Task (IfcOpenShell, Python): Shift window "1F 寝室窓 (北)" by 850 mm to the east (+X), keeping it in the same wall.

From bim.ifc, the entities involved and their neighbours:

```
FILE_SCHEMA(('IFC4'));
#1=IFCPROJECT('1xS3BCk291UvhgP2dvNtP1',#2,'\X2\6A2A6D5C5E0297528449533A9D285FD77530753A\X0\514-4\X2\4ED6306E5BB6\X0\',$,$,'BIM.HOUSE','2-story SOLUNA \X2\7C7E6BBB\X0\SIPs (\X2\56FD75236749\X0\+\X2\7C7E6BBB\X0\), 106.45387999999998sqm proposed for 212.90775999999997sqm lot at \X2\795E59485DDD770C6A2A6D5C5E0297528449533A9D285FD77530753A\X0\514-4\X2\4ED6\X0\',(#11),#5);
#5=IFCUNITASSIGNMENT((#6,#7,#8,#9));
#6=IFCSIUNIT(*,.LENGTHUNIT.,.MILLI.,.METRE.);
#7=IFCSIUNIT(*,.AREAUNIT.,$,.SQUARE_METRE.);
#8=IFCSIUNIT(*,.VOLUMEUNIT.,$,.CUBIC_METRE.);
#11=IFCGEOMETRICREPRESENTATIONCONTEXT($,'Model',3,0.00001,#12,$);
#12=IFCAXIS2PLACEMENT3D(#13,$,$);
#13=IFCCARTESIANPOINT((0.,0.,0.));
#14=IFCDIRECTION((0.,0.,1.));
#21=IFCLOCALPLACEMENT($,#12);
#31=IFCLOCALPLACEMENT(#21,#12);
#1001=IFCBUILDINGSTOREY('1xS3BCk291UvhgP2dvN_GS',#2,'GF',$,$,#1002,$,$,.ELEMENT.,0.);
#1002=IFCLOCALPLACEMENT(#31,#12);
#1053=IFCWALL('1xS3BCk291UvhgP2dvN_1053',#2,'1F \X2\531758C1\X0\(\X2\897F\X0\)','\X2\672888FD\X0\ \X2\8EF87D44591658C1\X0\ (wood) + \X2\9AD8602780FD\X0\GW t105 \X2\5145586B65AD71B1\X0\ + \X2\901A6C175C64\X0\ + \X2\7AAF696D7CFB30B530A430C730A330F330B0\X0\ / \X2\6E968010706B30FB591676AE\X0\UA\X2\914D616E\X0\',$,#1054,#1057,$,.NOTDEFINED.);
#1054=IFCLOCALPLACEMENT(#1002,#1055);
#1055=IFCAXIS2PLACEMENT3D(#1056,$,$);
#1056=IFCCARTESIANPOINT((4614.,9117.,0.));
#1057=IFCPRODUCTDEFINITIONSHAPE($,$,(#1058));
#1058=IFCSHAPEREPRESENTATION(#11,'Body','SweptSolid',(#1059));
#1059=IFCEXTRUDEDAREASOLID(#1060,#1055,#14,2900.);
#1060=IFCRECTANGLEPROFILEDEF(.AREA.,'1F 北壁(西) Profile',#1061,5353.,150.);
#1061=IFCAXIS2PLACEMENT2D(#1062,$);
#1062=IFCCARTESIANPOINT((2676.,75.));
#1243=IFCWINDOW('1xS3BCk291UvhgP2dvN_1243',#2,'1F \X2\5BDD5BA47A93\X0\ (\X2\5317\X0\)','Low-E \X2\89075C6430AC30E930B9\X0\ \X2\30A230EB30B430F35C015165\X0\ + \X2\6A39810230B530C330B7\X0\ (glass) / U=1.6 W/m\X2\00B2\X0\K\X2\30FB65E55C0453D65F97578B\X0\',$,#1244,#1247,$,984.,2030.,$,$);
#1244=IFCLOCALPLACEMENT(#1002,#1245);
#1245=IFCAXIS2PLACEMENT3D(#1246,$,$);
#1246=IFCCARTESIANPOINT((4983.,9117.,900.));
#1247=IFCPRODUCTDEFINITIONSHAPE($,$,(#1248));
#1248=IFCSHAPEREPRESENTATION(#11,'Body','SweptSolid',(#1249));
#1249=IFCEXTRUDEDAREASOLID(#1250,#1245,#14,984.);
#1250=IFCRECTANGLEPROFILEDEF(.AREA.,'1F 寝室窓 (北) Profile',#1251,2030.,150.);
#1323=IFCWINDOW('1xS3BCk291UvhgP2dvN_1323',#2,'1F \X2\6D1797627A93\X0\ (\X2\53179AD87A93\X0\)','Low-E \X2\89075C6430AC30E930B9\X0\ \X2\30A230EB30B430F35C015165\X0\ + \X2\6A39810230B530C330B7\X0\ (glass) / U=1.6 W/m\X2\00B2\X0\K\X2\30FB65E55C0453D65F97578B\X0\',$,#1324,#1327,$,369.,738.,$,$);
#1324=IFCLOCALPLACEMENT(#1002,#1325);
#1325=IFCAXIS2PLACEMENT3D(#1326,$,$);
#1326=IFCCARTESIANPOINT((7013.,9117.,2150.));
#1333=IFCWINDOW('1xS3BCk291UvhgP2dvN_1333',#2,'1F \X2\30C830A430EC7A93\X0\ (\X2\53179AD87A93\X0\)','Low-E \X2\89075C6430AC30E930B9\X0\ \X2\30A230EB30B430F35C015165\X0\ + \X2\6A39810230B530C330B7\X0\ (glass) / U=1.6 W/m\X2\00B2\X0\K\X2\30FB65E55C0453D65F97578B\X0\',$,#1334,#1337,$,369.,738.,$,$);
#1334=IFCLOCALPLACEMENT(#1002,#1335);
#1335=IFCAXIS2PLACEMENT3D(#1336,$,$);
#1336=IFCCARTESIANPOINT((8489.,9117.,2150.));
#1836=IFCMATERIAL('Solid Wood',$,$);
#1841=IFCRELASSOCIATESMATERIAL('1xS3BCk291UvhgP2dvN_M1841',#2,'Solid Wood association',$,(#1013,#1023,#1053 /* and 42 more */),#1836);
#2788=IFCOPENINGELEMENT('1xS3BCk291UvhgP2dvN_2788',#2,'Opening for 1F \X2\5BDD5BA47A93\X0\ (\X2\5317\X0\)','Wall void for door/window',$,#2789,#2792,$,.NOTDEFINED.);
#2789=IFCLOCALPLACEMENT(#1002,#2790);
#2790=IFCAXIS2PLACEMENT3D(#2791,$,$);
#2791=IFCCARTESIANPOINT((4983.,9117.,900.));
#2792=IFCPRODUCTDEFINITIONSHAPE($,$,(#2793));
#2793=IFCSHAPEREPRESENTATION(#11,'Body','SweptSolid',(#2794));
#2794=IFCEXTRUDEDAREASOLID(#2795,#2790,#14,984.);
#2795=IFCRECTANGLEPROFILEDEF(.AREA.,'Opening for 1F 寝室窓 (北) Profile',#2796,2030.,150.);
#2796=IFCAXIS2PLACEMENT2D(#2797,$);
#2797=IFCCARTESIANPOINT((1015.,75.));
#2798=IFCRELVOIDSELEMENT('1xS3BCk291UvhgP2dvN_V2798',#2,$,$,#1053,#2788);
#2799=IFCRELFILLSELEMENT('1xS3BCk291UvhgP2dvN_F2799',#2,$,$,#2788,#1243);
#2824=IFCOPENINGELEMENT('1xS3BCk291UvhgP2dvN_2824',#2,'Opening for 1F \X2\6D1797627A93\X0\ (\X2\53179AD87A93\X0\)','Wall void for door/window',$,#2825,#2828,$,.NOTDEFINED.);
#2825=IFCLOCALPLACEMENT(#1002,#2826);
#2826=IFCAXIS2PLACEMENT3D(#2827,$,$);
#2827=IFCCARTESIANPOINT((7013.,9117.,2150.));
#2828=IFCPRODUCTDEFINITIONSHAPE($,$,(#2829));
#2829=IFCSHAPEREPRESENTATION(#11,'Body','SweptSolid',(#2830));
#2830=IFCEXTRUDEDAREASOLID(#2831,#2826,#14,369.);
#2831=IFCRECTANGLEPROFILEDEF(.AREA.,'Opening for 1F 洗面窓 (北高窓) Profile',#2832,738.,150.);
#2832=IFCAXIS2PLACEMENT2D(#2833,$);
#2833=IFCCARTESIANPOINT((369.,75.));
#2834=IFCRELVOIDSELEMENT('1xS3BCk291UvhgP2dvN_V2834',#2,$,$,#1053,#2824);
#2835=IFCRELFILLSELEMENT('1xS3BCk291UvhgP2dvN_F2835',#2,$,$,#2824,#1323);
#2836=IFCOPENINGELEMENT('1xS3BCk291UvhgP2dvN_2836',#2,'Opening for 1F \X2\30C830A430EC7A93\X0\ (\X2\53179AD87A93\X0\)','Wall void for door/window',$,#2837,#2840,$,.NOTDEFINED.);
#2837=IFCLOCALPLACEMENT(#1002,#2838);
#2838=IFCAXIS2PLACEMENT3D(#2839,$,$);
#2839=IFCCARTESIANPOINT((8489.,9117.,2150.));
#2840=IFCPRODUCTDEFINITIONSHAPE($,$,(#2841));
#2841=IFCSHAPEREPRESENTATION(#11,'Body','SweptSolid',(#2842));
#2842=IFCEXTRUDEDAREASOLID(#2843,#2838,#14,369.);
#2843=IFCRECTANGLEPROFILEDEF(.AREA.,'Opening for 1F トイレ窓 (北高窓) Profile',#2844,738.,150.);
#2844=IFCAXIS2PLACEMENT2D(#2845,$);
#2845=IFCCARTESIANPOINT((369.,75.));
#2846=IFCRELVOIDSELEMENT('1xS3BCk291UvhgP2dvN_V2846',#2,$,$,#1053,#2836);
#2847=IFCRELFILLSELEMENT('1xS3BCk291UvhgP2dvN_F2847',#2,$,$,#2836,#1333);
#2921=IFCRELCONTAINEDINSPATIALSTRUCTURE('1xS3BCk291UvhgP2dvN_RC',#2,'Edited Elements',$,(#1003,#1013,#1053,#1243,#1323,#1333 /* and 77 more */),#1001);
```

```python
import ifcopenshell
import ifcopenshell.api.geometry
import ifcopenshell.util.placement
import ifcopenshell.util.unit

model = ifcopenshell.open("bim.ifc")
unit_scale = ifcopenshell.util.unit.calculate_unit_scale(model)

window = model.by_guid("1xS3BCk291UvhgP2dvN_1243")
opening = window.FillsVoids[0].RelatingOpeningElement
wall = opening.VoidsElements[0].RelatingBuildingElement

wall_matrix = ifcopenshell.util.placement.get_local_placement(wall.ObjectPlacement)
shift = wall_matrix[:3, 0] * 0.85 / unit_scale
before = ifcopenshell.util.placement.get_local_placement(window.ObjectPlacement)[:3, 3].copy()

# The window is not placed relative to its opening, so move both.
for product in (opening, window):
    matrix = ifcopenshell.util.placement.get_local_placement(product.ObjectPlacement)
    matrix[:3, 3] += shift
    ifcopenshell.api.geometry.edit_object_placement(model, product=product, matrix=matrix, is_si=False)

after = ifcopenshell.util.placement.get_local_placement(window.ObjectPlacement)[:3, 3]
print("window moved by", (after - before).round(3) + 0.0)

model.write("bim_v2.ifc")
```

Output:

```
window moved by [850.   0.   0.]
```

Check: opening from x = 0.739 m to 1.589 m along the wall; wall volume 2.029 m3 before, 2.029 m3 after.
